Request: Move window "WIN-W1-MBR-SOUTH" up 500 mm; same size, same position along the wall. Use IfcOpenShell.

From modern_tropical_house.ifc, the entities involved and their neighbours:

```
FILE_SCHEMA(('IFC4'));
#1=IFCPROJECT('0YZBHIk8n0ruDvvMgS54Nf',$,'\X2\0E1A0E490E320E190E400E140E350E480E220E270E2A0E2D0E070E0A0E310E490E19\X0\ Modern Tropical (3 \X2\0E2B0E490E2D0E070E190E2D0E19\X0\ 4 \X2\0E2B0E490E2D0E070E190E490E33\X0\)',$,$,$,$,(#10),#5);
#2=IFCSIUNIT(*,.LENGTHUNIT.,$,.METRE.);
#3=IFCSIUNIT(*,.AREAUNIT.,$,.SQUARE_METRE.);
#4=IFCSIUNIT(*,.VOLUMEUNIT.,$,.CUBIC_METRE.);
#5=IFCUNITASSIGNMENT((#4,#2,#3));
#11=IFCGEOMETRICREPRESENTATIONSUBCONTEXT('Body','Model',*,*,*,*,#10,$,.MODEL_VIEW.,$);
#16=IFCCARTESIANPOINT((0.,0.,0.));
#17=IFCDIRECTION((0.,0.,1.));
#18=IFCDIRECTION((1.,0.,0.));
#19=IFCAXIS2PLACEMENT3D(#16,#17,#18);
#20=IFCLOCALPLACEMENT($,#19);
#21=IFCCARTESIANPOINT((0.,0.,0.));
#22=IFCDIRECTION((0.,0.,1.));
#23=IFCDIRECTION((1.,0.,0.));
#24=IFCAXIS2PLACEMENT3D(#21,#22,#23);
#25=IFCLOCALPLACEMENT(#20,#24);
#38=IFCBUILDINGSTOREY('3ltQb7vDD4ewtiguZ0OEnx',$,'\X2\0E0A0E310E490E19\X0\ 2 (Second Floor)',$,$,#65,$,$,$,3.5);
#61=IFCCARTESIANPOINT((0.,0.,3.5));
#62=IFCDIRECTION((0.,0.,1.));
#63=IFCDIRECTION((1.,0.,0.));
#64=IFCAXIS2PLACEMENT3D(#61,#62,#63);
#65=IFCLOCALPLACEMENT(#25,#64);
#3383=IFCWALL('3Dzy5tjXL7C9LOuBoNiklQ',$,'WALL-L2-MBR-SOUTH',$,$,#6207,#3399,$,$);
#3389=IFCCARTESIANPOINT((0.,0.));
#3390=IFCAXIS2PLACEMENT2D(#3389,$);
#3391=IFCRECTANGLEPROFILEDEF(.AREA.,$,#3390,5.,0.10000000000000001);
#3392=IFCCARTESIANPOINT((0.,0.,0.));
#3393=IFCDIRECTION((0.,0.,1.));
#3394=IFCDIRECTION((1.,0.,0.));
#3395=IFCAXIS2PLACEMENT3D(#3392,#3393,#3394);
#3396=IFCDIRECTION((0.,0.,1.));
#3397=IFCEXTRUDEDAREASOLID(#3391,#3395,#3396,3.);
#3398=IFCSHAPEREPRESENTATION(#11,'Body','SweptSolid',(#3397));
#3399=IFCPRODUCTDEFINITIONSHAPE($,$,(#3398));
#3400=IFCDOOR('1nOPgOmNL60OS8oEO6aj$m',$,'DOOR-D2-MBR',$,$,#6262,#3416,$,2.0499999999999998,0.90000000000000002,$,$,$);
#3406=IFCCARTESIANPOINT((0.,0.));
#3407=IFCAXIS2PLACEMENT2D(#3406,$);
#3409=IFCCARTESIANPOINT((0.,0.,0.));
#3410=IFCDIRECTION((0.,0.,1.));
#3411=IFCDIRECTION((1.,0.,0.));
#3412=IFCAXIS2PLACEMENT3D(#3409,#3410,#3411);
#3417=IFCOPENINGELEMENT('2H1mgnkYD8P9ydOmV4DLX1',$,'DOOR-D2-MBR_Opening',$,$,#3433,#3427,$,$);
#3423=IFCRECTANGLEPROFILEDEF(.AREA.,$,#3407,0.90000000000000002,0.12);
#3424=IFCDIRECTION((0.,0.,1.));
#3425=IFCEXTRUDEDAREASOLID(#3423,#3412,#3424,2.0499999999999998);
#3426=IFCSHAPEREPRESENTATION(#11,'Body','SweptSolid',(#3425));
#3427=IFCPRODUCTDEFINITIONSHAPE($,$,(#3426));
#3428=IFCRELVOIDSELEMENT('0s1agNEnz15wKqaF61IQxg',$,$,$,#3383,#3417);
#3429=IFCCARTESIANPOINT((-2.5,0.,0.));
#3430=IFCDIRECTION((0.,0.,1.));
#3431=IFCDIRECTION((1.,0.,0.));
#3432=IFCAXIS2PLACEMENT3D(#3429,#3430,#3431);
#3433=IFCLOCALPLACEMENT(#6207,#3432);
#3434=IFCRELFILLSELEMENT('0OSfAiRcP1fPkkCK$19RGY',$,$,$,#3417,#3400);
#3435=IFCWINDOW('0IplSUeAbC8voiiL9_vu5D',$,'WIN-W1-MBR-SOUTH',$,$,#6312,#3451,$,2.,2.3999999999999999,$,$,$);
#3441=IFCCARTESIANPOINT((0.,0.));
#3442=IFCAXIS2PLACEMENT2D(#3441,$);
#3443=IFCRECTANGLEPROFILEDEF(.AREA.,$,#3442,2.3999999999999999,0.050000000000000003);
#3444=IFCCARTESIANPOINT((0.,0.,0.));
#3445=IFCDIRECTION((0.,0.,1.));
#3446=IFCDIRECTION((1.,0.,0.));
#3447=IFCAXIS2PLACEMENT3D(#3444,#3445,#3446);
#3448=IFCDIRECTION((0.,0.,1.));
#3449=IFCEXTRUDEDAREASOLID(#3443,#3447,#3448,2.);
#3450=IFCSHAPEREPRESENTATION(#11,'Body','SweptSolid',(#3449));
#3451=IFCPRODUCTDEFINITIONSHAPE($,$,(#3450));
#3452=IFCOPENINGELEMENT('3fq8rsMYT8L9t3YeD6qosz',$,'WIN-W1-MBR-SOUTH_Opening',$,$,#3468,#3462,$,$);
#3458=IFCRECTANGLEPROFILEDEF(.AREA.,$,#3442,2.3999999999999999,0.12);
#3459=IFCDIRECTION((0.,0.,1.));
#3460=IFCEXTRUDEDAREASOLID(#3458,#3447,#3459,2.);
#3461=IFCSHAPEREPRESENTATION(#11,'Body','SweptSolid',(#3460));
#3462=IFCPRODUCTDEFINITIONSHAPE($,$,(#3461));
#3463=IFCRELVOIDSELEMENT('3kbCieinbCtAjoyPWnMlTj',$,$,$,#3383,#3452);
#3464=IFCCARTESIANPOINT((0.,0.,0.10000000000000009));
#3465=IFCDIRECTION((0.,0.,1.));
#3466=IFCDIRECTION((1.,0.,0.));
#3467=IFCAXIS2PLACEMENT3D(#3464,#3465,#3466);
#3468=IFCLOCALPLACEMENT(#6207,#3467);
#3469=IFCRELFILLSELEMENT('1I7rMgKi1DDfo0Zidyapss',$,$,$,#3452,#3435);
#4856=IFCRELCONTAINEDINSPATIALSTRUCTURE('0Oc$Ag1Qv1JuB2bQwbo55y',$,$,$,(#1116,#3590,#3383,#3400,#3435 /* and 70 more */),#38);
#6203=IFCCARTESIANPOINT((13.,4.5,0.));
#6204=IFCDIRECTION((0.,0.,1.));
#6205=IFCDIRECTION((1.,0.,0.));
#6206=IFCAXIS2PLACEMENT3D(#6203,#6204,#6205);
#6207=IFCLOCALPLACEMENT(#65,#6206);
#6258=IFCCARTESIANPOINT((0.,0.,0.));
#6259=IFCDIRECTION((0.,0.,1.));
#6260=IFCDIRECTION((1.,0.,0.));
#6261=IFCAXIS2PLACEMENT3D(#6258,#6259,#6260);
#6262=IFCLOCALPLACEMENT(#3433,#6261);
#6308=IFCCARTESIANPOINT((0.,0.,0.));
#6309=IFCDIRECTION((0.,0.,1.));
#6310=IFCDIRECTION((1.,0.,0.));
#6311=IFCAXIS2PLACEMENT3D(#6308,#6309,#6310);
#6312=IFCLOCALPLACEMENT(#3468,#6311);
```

```python
import numpy as np
import ifcopenshell
import ifcopenshell.api.geometry
import ifcopenshell.util.placement
import ifcopenshell.util.unit

model = ifcopenshell.open("modern_tropical_house.ifc")
unit_scale = ifcopenshell.util.unit.calculate_unit_scale(model)

window = model.by_id(3435)
opening = window.FillsVoids[0].RelatingOpeningElement
dz = 0.5

shift = np.array([0.0, 0.0, dz])
# The window is placed relative to its opening, so it follows when the opening moves.
matrix = ifcopenshell.util.placement.get_local_placement(opening.ObjectPlacement)
matrix[:3, 3] += shift
ifcopenshell.api.geometry.edit_object_placement(
    model, product=opening, matrix=matrix, is_si=False, should_transform_children=True
)

print(f"moved by {dz * unit_scale:+.3f} m")

model.write("modern_tropical_house_v2.ifc")
```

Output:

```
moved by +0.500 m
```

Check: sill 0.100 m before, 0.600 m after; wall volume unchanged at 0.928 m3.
